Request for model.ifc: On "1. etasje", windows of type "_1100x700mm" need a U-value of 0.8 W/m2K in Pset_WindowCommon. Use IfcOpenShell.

First a look at what the model holds.

```python
import ifcopenshell
import ifcopenshell.util.element

model = ifcopenshell.open("model.ifc")
print(model.schema)
storey = next(s for s in model.by_type("IfcBuildingStorey") if s.Name == "1. etasje")
windows = [e for e in ifcopenshell.util.element.get_decomposition(storey) if e.is_a("IfcWindow")]
seen = {}
for e in windows:
    element_type = ifcopenshell.util.element.get_type(e)
    key = (element_type.Name if element_type != e and element_type else None, ifcopenshell.util.element.get_pset(e, "Pset_WindowCommon", "ThermalTransmittance"))
    seen[key] = seen.get(key, 0) + 1
for (name, value), count in sorted(seen.items(), key=str):
    print(count, "x", name, "|", value)
```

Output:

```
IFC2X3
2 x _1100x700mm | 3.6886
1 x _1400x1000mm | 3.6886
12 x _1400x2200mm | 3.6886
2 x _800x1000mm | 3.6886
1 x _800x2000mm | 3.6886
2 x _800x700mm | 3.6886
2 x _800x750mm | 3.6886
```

```python
import ifcopenshell
import ifcopenshell.api.pset
import ifcopenshell.util.element

model = ifcopenshell.open("model.ifc")

storey = next(s for s in model.by_type("IfcBuildingStorey") if s.Name == "1. etasje")
windows = [e for e in ifcopenshell.util.element.get_decomposition(storey) if e.is_a("IfcWindow")]

count = 0
for e in windows:
    element_type = ifcopenshell.util.element.get_type(e)
    if element_type in (None, e) or element_type.Name != "_1100x700mm":
        continue
    # add_pset returns the element's existing set when there is one.
    pset = ifcopenshell.api.pset.add_pset(model, product=e, name="Pset_WindowCommon")
    ifcopenshell.api.pset.edit_pset(model, pset=pset, properties={"ThermalTransmittance": 0.8})
    count += 1

print(count, "windows updated")

model.write("model_edited.ifc")
```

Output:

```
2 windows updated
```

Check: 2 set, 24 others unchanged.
